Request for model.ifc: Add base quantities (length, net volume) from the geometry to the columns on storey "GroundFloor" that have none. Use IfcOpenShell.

First a look at what the model holds.

```python
import ifcopenshell
import ifcopenshell.util.element
import ifcopenshell.util.unit

model = ifcopenshell.open("model.ifc")
print(model.schema)
for unit_type in ("LENGTHUNIT", "AREAUNIT", "VOLUMEUNIT"):
    print(unit_type, ifcopenshell.util.unit.calculate_unit_scale(model, unit_type))
storey = next(s for s in model.by_type("IfcBuildingStorey") if s.Name == "GroundFloor")
columns = [e for e in ifcopenshell.util.element.get_decomposition(storey) if e.is_a("IfcColumn")]
for e in sorted(columns, key=lambda e: e.id()):
    print(e.id(), e.is_a(), e.Name, list(ifcopenshell.util.element.get_psets(e, qtos_only=True)), sep=" | ")
```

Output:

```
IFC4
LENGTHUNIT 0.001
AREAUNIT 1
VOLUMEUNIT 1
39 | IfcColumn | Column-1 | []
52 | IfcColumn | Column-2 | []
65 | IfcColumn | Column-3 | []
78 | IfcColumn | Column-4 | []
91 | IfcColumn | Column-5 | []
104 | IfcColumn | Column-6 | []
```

```python
import ifcopenshell
import ifcopenshell.api.pset
import ifcopenshell.geom
import ifcopenshell.util.element
import ifcopenshell.util.shape
import ifcopenshell.util.unit

model = ifcopenshell.open("model.ifc")
unit_scale = ifcopenshell.util.unit.calculate_unit_scale(model)
volume_scale = ifcopenshell.util.unit.calculate_unit_scale(model, "VOLUMEUNIT")
settings = ifcopenshell.geom.settings()

storey = next(s for s in model.by_type("IfcBuildingStorey") if s.Name == "GroundFloor")
columns = [e for e in ifcopenshell.util.element.get_decomposition(storey) if e.is_a("IfcColumn")]

for e in sorted(columns, key=lambda e: e.id()):
    if ifcopenshell.util.element.get_psets(e, qtos_only=True, should_inherit=False):
        continue
    # Geometry comes back in metres, in the element's own axes.
    shape = ifcopenshell.geom.create_shape(settings, e)
    values = {
        "Length": ifcopenshell.util.shape.get_z(shape.geometry) / unit_scale,
        "NetVolume": ifcopenshell.util.shape.get_volume(shape.geometry) / volume_scale,
    }
    qto = ifcopenshell.api.pset.add_qto(model, product=e, name="Qto_ColumnBaseQuantities")
    ifcopenshell.api.pset.edit_qto(model, qto=qto, properties=values)
    print(e.id(), {k: round(v, 3) for k, v in values.items()})

model.write("model_rev.ifc")
```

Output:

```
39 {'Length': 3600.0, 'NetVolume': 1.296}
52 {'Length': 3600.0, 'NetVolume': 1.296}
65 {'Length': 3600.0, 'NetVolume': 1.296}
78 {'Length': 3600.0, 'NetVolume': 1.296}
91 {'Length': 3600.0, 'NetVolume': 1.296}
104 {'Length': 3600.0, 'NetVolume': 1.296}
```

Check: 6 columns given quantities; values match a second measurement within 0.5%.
